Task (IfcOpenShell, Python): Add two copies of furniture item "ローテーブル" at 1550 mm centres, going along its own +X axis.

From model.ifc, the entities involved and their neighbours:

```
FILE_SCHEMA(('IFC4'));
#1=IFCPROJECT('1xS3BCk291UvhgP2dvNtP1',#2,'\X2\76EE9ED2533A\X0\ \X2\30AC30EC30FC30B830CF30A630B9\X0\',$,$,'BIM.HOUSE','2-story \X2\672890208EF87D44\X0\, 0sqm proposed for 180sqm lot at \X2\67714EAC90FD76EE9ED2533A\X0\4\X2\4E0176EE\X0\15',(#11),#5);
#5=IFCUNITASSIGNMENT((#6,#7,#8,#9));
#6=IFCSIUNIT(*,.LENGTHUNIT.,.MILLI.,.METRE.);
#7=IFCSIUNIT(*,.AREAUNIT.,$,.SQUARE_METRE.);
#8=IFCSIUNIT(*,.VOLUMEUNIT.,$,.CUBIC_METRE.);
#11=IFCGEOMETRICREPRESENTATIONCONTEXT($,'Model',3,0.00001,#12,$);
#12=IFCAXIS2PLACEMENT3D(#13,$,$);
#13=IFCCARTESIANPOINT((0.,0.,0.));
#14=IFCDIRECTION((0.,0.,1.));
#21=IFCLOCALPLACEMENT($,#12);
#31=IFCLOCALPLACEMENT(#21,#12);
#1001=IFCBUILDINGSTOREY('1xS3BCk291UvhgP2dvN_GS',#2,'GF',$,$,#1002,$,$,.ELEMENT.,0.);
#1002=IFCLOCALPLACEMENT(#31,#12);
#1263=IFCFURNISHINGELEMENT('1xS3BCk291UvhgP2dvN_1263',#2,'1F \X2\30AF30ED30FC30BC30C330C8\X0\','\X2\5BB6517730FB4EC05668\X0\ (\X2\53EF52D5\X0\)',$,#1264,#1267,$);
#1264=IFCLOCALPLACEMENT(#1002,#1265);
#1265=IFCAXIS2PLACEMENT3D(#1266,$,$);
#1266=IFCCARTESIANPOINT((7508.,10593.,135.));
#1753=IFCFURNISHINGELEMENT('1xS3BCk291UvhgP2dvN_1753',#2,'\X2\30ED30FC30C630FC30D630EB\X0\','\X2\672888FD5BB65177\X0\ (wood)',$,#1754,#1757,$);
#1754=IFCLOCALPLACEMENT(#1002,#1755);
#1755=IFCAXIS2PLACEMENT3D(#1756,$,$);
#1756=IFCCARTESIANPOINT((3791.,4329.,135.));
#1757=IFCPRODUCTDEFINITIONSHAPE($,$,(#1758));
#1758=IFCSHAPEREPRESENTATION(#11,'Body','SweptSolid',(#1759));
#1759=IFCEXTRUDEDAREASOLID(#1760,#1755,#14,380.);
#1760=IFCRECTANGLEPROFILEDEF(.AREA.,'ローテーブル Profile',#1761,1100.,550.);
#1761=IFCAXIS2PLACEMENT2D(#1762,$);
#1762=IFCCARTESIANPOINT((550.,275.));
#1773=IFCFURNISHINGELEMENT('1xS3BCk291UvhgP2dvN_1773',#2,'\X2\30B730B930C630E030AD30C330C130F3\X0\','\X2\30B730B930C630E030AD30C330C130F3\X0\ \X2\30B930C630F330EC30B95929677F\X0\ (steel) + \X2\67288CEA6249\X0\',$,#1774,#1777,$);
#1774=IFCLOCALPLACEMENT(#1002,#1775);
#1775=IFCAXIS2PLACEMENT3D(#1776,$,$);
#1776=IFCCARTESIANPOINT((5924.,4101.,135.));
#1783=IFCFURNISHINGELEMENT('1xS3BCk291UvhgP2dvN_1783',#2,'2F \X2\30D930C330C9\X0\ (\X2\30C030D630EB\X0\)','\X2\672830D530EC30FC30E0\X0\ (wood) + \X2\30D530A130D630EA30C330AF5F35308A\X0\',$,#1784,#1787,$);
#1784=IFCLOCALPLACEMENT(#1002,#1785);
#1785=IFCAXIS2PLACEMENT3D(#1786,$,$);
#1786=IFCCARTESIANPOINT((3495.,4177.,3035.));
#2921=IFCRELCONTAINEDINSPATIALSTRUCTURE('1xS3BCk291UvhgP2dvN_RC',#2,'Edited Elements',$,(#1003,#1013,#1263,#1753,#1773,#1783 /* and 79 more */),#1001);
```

```python
import ifcopenshell
import ifcopenshell.api.geometry
import ifcopenshell.api.root
import ifcopenshell.util.element
import ifcopenshell.util.placement
import ifcopenshell.util.unit

model = ifcopenshell.open("model.ifc")
unit_scale = ifcopenshell.util.unit.calculate_unit_scale(model)


def reuse_history(source, copy):
    """copy_class also copies each property set's owner history, people and application; keep the originals."""
    for rel in copy.IsDefinedBy:
        if rel.is_a("IfcRelDefinesByProperties") and (history := rel.RelatingPropertyDefinition.OwnerHistory):
            rel.RelatingPropertyDefinition.OwnerHistory = source.OwnerHistory
            ifcopenshell.util.element.remove_deep2(model, history)


source = model.by_guid("1xS3BCk291UvhgP2dvN_1753")
base = ifcopenshell.util.placement.get_local_placement(source.ObjectPlacement)
step = base[:3, 0] * 1.55 / unit_scale

for i in range(1, 3):
    copy = ifcopenshell.api.root.copy_class(model, product=source)
    copy.Representation = ifcopenshell.util.element.copy_deep(
        model, source.Representation, exclude=["IfcGeometricRepresentationContext", "IfcRepresentationMap"]
    )
    reuse_history(source, copy)
    matrix = base.copy()
    matrix[:3, 3] += i * step
    print("added at", matrix[:3, 3].round(3) + 0.0)
    ifcopenshell.api.geometry.edit_object_placement(model, product=copy, matrix=matrix, is_si=False)

model.write("model-out.ifc")
```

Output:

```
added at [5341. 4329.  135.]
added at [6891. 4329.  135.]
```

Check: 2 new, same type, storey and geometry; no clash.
